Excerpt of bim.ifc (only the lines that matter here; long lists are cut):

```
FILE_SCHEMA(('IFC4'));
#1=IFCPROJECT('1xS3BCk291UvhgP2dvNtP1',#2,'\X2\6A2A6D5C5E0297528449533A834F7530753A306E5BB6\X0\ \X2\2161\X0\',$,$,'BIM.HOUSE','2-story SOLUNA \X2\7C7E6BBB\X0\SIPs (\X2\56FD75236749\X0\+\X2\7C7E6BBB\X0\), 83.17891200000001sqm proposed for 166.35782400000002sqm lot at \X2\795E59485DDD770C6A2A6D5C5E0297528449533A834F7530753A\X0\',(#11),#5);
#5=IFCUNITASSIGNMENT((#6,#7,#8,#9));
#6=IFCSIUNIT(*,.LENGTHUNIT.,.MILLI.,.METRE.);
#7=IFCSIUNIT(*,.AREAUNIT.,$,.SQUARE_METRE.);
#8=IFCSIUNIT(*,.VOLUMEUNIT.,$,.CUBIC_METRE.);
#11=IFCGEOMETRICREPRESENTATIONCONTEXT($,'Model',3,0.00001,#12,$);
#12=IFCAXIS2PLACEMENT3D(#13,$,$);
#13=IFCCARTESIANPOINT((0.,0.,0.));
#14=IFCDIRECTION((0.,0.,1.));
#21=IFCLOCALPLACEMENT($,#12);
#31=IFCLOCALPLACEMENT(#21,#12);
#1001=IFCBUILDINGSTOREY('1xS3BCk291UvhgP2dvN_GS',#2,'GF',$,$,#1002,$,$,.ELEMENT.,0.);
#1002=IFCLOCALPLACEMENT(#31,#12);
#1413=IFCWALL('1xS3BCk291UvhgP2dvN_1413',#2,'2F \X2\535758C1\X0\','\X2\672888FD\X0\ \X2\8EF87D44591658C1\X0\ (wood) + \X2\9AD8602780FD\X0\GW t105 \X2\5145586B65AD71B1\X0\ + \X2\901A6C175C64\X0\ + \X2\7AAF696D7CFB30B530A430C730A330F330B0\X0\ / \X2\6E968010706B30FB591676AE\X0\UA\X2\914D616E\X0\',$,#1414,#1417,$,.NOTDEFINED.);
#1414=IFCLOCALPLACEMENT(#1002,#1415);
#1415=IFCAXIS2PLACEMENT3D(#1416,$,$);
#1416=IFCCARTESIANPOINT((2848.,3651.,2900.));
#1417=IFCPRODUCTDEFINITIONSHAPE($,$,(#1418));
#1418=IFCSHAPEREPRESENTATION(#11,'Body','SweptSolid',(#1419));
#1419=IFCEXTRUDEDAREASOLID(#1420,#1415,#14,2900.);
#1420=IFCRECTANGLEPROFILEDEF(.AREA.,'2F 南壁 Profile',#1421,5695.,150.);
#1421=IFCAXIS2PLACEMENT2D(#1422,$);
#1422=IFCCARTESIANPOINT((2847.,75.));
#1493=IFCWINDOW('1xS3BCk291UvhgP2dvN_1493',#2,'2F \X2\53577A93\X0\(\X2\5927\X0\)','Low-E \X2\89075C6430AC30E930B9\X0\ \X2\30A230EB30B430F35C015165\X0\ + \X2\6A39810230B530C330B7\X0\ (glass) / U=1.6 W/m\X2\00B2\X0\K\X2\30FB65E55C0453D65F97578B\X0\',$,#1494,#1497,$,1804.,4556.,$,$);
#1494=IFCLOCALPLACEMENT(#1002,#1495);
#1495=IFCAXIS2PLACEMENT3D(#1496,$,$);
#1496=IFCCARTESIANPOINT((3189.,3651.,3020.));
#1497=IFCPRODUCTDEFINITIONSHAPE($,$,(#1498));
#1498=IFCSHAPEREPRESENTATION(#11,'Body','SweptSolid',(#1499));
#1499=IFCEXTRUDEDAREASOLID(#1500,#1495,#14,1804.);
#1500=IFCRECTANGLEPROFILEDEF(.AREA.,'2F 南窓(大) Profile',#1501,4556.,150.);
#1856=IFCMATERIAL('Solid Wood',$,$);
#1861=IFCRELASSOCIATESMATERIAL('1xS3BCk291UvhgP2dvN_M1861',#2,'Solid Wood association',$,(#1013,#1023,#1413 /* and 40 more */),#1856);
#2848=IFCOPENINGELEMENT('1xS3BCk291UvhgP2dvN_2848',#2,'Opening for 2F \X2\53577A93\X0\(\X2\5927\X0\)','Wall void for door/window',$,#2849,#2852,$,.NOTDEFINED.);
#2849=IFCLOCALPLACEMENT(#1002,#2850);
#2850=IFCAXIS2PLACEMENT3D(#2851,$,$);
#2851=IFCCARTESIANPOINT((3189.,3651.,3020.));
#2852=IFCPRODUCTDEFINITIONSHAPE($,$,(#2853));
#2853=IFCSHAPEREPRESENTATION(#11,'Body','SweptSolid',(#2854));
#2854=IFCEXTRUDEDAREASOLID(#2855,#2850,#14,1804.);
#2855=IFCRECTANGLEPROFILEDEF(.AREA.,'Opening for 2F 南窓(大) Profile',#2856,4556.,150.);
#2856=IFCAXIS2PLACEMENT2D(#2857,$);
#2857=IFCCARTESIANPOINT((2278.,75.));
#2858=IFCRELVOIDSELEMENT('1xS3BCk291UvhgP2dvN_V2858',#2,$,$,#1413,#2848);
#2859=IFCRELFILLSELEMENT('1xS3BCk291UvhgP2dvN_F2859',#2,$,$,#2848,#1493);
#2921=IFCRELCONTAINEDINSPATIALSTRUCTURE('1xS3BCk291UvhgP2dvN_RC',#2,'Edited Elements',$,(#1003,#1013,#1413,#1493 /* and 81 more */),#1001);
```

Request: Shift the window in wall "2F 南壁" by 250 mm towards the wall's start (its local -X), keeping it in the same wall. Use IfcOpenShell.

```python
import ifcopenshell
import ifcopenshell.api.geometry
import ifcopenshell.util.placement
import ifcopenshell.util.unit

model = ifcopenshell.open("bim.ifc")
unit_scale = ifcopenshell.util.unit.calculate_unit_scale(model)

window = model.by_guid("1xS3BCk291UvhgP2dvN_1493")
opening = window.FillsVoids[0].RelatingOpeningElement
wall = opening.VoidsElements[0].RelatingBuildingElement

wall_matrix = ifcopenshell.util.placement.get_local_placement(wall.ObjectPlacement)
shift = wall_matrix[:3, 0] * -0.25 / unit_scale
before = ifcopenshell.util.placement.get_local_placement(window.ObjectPlacement)[:3, 3].copy()

# The window is not placed relative to its opening, so move both.
for product in (opening, window):
    matrix = ifcopenshell.util.placement.get_local_placement(product.ObjectPlacement)
    matrix[:3, 3] += shift
    ifcopenshell.api.geometry.edit_object_placement(model, product=product, matrix=matrix, is_si=False)

after = ifcopenshell.util.placement.get_local_placement(window.ObjectPlacement)[:3, 3]
print("window moved by", (after - before).round(3) + 0.0)

model.write("bim_updated.ifc")
```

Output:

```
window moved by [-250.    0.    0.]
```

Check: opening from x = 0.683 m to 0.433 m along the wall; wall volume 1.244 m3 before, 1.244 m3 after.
